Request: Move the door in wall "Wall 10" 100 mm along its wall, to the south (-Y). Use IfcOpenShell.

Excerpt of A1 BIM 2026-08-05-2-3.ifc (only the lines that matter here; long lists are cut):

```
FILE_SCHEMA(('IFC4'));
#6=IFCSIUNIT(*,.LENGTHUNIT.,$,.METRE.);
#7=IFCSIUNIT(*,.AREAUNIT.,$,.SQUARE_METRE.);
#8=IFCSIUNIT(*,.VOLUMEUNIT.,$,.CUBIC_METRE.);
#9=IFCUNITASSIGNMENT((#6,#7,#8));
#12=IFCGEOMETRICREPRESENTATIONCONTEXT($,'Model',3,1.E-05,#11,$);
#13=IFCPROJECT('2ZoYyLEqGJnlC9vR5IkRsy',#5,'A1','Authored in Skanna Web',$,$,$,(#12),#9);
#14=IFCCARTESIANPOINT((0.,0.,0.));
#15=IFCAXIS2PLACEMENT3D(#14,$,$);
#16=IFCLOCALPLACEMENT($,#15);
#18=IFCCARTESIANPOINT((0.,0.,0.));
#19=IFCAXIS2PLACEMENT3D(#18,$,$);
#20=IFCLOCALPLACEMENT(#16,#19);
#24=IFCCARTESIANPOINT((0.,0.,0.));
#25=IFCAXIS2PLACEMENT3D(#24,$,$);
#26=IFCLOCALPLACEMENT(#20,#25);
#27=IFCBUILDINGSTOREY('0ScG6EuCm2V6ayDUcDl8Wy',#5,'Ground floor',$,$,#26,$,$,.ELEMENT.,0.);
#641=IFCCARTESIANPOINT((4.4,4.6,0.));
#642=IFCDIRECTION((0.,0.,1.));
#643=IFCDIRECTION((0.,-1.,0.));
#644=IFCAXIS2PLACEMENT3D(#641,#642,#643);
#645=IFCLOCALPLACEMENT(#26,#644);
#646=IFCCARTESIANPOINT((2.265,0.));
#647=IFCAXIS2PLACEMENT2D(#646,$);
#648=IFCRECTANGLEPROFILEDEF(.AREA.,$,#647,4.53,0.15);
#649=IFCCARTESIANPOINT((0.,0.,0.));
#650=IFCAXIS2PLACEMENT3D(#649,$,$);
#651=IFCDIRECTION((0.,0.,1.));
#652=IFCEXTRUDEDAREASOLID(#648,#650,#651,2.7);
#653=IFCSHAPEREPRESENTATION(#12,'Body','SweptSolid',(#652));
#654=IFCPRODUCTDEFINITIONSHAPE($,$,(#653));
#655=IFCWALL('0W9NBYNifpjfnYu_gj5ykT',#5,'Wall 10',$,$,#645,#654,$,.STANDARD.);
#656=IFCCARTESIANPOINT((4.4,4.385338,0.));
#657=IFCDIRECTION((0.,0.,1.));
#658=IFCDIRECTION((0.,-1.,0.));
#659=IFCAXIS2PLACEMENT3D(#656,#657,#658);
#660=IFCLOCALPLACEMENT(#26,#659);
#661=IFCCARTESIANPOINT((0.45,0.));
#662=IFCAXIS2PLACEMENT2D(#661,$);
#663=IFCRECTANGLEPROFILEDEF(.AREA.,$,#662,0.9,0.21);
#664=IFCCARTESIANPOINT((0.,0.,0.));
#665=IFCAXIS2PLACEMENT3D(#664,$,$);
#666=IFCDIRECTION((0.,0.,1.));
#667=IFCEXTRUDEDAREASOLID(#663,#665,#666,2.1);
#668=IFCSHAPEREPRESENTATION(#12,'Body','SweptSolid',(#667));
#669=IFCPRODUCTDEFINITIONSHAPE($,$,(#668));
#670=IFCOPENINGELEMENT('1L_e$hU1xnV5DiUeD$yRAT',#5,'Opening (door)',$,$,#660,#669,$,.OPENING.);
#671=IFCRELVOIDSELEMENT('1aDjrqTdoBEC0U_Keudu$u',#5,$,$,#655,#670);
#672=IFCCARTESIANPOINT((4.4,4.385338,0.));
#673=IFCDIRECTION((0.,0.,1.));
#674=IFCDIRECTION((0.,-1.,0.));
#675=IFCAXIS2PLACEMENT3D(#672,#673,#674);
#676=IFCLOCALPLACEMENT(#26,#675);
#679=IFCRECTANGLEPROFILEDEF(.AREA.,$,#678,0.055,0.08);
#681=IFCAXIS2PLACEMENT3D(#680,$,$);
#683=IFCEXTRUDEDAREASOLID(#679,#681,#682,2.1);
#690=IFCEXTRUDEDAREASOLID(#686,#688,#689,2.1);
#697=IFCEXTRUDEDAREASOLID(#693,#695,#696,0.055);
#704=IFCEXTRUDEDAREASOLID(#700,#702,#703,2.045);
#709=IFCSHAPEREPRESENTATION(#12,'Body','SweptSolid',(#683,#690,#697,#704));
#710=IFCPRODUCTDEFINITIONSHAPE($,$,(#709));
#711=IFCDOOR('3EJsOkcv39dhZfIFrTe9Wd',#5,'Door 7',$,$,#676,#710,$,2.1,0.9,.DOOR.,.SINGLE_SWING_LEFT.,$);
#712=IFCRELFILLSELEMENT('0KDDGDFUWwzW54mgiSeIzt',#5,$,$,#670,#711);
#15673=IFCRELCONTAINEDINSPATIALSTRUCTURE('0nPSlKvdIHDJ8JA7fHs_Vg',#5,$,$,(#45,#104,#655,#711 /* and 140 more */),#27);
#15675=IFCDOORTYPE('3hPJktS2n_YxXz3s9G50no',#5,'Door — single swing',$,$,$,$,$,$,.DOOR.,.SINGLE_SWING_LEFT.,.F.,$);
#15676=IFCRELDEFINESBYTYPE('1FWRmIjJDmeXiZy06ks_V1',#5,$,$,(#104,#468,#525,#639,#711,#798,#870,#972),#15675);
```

```python
import ifcopenshell
import ifcopenshell.api.geometry
import ifcopenshell.util.placement
import ifcopenshell.util.unit

model = ifcopenshell.open("A1 BIM 2026-08-05-2-3.ifc")
unit_scale = ifcopenshell.util.unit.calculate_unit_scale(model)

door = model.by_guid("3EJsOkcv39dhZfIFrTe9Wd")
opening = door.FillsVoids[0].RelatingOpeningElement
wall = opening.VoidsElements[0].RelatingBuildingElement

wall_matrix = ifcopenshell.util.placement.get_local_placement(wall.ObjectPlacement)
shift = wall_matrix[:3, 0] * 0.1 / unit_scale
before = ifcopenshell.util.placement.get_local_placement(door.ObjectPlacement)[:3, 3].copy()

# The door is not placed relative to its opening, so move both.
for product in (opening, door):
    matrix = ifcopenshell.util.placement.get_local_placement(product.ObjectPlacement)
    matrix[:3, 3] += shift
    ifcopenshell.api.geometry.edit_object_placement(model, product=product, matrix=matrix, is_si=False)

after = ifcopenshell.util.placement.get_local_placement(door.ObjectPlacement)[:3, 3]
print("door moved by", (after - before).round(3) + 0.0)

model.write("A1 BIM 2026-08-05-2-3_rev.ifc")
```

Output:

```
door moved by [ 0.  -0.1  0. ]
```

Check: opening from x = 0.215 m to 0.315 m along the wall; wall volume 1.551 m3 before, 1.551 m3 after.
